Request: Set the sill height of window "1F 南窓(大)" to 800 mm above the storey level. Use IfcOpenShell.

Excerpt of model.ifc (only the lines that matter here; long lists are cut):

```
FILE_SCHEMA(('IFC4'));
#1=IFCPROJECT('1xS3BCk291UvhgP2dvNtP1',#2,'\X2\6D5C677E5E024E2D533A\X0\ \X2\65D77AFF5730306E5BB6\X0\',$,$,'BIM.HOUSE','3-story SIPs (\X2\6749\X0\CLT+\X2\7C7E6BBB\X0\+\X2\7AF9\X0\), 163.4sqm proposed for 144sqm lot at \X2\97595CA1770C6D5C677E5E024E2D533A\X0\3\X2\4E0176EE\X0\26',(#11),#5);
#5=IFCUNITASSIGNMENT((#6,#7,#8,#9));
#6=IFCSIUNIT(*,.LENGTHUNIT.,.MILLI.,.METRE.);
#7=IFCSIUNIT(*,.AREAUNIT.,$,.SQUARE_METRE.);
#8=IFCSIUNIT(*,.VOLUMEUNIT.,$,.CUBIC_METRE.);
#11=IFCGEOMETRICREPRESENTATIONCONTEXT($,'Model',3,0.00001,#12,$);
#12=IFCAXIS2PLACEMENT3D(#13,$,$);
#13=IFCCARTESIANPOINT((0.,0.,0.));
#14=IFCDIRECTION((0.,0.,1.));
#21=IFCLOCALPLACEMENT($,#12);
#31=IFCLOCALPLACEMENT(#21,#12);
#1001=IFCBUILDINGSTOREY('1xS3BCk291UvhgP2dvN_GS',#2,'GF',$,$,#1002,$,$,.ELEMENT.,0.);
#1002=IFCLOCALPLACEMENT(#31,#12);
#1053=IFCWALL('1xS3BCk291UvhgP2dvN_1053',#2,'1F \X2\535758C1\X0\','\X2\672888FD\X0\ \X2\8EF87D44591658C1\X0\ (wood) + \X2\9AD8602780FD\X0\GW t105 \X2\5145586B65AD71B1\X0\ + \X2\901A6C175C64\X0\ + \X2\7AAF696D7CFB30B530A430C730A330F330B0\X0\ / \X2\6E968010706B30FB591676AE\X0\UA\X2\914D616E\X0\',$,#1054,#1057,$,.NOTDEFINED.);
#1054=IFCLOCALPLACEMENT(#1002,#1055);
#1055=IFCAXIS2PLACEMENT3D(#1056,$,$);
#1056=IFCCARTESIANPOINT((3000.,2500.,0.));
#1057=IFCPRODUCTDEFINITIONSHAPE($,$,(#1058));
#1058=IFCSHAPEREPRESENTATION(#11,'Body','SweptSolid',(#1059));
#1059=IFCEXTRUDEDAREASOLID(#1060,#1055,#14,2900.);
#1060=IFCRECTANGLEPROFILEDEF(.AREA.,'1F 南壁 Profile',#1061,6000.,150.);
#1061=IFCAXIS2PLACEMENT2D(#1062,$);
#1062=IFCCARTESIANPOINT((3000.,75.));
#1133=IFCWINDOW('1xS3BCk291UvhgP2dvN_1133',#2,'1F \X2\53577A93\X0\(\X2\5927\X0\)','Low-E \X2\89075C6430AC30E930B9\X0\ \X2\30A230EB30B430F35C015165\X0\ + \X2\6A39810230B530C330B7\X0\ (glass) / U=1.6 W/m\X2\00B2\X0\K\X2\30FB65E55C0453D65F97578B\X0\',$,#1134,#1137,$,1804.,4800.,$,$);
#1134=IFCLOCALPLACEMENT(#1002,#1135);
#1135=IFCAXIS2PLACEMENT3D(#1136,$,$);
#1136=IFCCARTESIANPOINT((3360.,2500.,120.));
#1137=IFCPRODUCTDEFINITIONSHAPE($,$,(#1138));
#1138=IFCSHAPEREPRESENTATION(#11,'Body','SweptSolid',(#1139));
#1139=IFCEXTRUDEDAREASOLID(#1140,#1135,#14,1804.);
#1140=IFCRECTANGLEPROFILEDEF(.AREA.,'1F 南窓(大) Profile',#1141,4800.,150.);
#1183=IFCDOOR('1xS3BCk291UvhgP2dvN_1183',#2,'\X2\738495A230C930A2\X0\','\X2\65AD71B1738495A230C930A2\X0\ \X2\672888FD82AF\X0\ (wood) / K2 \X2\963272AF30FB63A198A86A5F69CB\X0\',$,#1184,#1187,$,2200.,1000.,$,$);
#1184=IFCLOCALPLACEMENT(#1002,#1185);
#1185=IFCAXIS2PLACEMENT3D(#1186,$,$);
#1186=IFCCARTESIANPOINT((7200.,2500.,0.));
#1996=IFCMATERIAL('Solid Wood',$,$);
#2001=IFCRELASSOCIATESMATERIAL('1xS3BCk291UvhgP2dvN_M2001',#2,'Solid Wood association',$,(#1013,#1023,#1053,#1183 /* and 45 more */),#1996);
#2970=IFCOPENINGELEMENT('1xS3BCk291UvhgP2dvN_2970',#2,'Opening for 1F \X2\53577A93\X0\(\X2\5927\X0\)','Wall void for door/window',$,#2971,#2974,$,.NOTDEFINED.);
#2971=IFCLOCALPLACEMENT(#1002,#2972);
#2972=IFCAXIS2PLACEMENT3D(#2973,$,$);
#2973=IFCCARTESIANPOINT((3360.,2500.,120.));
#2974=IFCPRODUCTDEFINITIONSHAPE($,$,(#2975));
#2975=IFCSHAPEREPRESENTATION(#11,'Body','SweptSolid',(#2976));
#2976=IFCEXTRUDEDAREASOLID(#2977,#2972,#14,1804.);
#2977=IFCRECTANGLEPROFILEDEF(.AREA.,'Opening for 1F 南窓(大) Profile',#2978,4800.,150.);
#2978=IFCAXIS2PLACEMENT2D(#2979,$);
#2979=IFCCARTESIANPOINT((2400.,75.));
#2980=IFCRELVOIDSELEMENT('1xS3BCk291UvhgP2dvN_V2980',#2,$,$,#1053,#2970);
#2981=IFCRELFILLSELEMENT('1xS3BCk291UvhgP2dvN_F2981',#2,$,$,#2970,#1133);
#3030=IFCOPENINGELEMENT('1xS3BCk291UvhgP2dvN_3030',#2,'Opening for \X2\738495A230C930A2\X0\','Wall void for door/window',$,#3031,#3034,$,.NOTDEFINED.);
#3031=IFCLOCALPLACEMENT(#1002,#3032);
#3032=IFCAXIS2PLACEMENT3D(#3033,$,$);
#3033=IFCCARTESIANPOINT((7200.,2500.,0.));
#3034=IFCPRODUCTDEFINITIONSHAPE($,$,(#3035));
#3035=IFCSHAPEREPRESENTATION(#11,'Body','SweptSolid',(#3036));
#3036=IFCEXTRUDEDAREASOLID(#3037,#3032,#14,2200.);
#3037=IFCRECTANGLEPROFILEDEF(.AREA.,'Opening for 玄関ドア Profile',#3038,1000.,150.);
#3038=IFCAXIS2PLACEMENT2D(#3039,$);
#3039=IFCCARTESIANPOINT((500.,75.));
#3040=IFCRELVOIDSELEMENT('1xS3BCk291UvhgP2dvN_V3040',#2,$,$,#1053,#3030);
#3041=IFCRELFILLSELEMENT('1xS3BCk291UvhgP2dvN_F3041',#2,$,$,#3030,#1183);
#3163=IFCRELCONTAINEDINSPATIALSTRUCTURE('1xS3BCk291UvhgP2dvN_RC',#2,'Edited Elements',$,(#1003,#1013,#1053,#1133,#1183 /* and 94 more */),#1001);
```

```python
import numpy as np
import ifcopenshell
import ifcopenshell.api.geometry
import ifcopenshell.geom
import ifcopenshell.util.element
import ifcopenshell.util.placement
import ifcopenshell.util.shape
import ifcopenshell.util.unit

model = ifcopenshell.open("model.ifc")
unit_scale = ifcopenshell.util.unit.calculate_unit_scale(model)

window = model.by_id(1133)
opening = window.FillsVoids[0].RelatingOpeningElement
storey = ifcopenshell.util.element.get_container(window, ifc_class="IfcBuildingStorey")
level = ifcopenshell.util.placement.get_local_placement(storey.ObjectPlacement)[2, 3]

# The opening's origin need not be at the sill, so measure its lowest point.
shape = ifcopenshell.geom.create_shape(ifcopenshell.geom.settings(), opening)
bottom = ifcopenshell.util.shape.get_shape_bottom_elevation(shape, shape.geometry) / unit_scale
dz = level + 0.8 / unit_scale - bottom

shift = np.array([0.0, 0.0, dz])
# The window is not placed relative to its opening, so move both.
for product in (opening, window):
    matrix = ifcopenshell.util.placement.get_local_placement(product.ObjectPlacement)
    matrix[:3, 3] += shift
    ifcopenshell.api.geometry.edit_object_placement(model, product=product, matrix=matrix, is_si=False)

print(f"moved by {dz * unit_scale:+.3f} m")

model.write("model_edited.ifc")
```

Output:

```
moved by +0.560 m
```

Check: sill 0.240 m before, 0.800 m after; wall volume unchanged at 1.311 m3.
